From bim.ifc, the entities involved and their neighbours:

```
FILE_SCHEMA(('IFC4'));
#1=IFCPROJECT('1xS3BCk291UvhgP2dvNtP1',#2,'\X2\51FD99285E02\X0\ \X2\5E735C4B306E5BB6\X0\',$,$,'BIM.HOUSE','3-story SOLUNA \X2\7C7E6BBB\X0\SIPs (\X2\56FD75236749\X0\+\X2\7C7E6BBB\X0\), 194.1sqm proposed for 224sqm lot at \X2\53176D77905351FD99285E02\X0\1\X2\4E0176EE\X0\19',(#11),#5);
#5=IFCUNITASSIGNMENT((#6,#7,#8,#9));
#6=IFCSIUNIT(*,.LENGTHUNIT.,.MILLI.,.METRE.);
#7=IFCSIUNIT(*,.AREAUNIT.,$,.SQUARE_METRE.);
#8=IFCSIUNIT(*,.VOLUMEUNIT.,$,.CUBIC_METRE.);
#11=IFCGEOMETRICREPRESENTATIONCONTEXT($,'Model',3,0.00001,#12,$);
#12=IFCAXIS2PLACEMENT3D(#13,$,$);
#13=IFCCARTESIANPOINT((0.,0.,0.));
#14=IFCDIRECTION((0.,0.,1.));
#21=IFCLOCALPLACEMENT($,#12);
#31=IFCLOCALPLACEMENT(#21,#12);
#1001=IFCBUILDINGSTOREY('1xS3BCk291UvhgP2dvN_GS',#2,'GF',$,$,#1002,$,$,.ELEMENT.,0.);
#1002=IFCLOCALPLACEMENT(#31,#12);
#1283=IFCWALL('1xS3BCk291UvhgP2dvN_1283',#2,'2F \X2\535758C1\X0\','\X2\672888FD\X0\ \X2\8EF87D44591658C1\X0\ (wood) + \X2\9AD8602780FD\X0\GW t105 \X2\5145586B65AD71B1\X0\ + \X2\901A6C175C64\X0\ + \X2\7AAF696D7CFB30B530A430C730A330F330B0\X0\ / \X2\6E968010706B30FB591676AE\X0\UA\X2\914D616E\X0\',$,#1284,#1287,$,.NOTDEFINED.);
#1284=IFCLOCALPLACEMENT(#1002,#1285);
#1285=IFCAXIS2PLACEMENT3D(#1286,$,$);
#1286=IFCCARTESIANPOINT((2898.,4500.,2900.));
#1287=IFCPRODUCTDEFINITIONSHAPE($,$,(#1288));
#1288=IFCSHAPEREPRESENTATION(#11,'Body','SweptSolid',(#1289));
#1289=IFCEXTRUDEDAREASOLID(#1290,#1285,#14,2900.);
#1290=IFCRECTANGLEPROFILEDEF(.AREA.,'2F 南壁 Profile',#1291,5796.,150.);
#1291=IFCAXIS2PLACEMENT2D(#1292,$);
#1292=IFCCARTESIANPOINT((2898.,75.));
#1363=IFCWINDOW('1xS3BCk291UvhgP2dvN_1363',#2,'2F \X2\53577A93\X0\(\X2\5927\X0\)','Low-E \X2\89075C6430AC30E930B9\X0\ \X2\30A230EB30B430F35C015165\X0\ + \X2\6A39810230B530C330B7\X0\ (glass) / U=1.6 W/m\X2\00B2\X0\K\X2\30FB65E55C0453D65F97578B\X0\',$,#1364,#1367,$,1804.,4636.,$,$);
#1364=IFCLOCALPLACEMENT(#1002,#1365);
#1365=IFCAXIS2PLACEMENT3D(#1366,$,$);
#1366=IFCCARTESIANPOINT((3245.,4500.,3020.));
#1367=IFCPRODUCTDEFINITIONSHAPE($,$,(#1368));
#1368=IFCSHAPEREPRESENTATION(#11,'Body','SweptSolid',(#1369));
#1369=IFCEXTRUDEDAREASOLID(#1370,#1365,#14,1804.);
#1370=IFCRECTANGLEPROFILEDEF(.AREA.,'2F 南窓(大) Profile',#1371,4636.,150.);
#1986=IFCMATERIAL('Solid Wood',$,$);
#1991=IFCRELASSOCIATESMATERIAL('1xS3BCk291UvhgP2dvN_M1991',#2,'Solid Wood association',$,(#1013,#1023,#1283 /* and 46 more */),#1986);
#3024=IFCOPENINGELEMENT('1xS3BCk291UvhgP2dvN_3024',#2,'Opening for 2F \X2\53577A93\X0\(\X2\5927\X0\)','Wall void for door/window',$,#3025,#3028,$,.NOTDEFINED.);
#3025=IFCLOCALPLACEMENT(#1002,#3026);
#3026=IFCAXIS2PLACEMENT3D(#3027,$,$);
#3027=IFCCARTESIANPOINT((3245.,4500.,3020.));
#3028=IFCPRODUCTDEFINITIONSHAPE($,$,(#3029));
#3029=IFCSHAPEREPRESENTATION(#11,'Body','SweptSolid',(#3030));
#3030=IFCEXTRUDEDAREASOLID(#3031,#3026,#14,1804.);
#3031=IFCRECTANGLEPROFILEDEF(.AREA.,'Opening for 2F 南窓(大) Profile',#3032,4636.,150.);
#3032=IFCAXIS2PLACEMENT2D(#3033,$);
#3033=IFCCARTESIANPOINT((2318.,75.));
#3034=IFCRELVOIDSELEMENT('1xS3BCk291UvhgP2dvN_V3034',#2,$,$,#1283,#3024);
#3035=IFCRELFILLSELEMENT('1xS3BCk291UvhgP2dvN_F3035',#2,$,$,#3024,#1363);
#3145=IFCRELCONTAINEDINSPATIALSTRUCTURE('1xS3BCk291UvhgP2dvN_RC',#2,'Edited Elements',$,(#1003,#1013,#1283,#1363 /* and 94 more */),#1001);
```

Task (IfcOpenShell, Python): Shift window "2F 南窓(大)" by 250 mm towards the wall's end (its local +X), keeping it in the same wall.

```python
import ifcopenshell
import ifcopenshell.api.geometry
import ifcopenshell.util.placement

model = ifcopenshell.open("bim.ifc")

window = model.by_guid("1xS3BCk291UvhgP2dvN_1363")
opening = window.FillsVoids[0].RelatingOpeningElement
wall = opening.VoidsElements[0].RelatingBuildingElement

wall_matrix = ifcopenshell.util.placement.get_local_placement(wall.ObjectPlacement)
shift = wall_matrix[:3, 0] * 250.0
before = ifcopenshell.util.placement.get_local_placement(window.ObjectPlacement)[:3, 3].copy()

# The window is not placed relative to its opening, so move both.
for product in (opening, window):
    matrix = ifcopenshell.util.placement.get_local_placement(product.ObjectPlacement)
    matrix[:3, 3] += shift
    ifcopenshell.api.geometry.edit_object_placement(model, product=product, matrix=matrix, is_si=False)

after = ifcopenshell.util.placement.get_local_placement(window.ObjectPlacement)[:3, 3]
print("window moved by", (after - before).round(3) + 0.0)

model.write("bim_v2.ifc")
```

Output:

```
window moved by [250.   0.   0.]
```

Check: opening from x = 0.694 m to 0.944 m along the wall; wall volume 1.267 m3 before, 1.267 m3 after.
